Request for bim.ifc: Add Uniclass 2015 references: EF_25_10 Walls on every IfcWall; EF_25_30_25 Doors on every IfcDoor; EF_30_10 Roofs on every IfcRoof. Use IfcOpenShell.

First a look at what the model holds.

```python
import ifcopenshell

model = ifcopenshell.open("bim.ifc")
print(model.schema)
print("classifications:", [c.Name for c in model.by_type("IfcClassification")])
for ifc_class in ("IfcDoor", "IfcRoof", "IfcStair", "IfcWall", "IfcWindow"):
    print(ifc_class, len(model.by_type(ifc_class)))
```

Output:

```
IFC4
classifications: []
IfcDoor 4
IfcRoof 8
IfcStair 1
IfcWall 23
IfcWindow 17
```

```python
import ifcopenshell
import ifcopenshell.api.classification

model = ifcopenshell.open("bim.ifc")

system = ifcopenshell.api.classification.add_classification(model, classification="Uniclass 2015")

codes = {
    "IfcWall": ("EF_25_10", "Walls"),
    "IfcDoor": ("EF_25_30_25", "Doors"),
    "IfcRoof": ("EF_30_10", "Roofs"),
}
for ifc_class, (code, name) in codes.items():
    products = model.by_type(ifc_class)
    ifcopenshell.api.classification.add_reference(
        model, products=products, classification=system, identification=code, name=name
    )
    print(code, len(products))

model.write("bim_updated.ifc")
```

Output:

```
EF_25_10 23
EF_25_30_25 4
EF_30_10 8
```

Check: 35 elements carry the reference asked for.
